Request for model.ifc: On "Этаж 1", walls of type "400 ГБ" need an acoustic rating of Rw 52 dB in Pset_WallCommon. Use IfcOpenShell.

First a look at what the model holds.

```python
import ifcopenshell
import ifcopenshell.util.element

model = ifcopenshell.open("model.ifc")
print(model.schema)
storey = next(s for s in model.by_type("IfcBuildingStorey") if s.Name == "Этаж 1")
walls = [e for e in ifcopenshell.util.element.get_decomposition(storey) if e.is_a("IfcWall")]
seen = {}
for e in walls:
    element_type = ifcopenshell.util.element.get_type(e)
    key = (element_type.Name if element_type != e and element_type else None, ifcopenshell.util.element.get_pset(e, "Pset_WallCommon", "AcousticRating"))
    seen[key] = seen.get(key, 0) + 1
for (name, value), count in sorted(seen.items(), key=str):
    print(count, "x", name, "|", value)
```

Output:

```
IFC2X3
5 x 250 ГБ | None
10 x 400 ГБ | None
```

```python
import ifcopenshell
import ifcopenshell.api.pset
import ifcopenshell.util.element

model = ifcopenshell.open("model.ifc")

storey = next(s for s in model.by_type("IfcBuildingStorey") if s.Name == "Этаж 1")
walls = [e for e in ifcopenshell.util.element.get_decomposition(storey) if e.is_a("IfcWall")]

count = 0
for e in walls:
    element_type = ifcopenshell.util.element.get_type(e)
    if element_type in (None, e) or element_type.Name != "400 ГБ":
        continue
    # add_pset returns the element's existing set when there is one.
    pset = ifcopenshell.api.pset.add_pset(model, product=e, name="Pset_WallCommon")
    ifcopenshell.api.pset.edit_pset(model, pset=pset, properties={"AcousticRating": "Rw 52 dB"})
    count += 1

print(count, "walls updated")

model.write("model-out.ifc")
```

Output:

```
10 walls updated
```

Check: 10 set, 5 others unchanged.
